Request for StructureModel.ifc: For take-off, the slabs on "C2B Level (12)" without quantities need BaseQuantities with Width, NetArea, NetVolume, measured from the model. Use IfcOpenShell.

First a look at what the model holds.

```python
import ifcopenshell
import ifcopenshell.util.element
import ifcopenshell.util.unit

model = ifcopenshell.open("StructureModel.ifc")
print(model.schema)
for unit_type in ("LENGTHUNIT", "AREAUNIT", "VOLUMEUNIT"):
    print(unit_type, ifcopenshell.util.unit.calculate_unit_scale(model, unit_type))
storey = next(s for s in model.by_type("IfcBuildingStorey") if s.Name == "C2B Level (12)")
slabs = [e for e in ifcopenshell.util.element.get_decomposition(storey) if e.is_a("IfcSlab")]
for e in sorted(slabs, key=lambda e: e.id()):
    print(e.id(), e.is_a(), e.Name, list(ifcopenshell.util.element.get_psets(e, qtos_only=True)), sep=" | ")
```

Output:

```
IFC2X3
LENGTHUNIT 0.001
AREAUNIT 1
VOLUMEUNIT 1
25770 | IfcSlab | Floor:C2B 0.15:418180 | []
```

```python
import ifcopenshell
import ifcopenshell.api.pset
import ifcopenshell.geom
import ifcopenshell.util.element
import ifcopenshell.util.shape
import ifcopenshell.util.unit

model = ifcopenshell.open("StructureModel.ifc")
unit_scale = ifcopenshell.util.unit.calculate_unit_scale(model)
area_scale = ifcopenshell.util.unit.calculate_unit_scale(model, "AREAUNIT")
volume_scale = ifcopenshell.util.unit.calculate_unit_scale(model, "VOLUMEUNIT")
settings = ifcopenshell.geom.settings()

storey = next(s for s in model.by_type("IfcBuildingStorey") if s.Name == "C2B Level (12)")
slabs = [e for e in ifcopenshell.util.element.get_decomposition(storey) if e.is_a("IfcSlab")]

for e in sorted(slabs, key=lambda e: e.id()):
    if ifcopenshell.util.element.get_psets(e, qtos_only=True, should_inherit=False):
        continue
    # Geometry comes back in metres, in the element's own axes.
    shape = ifcopenshell.geom.create_shape(settings, e)
    values = {
        "Width": ifcopenshell.util.shape.get_z(shape.geometry) / unit_scale,
        "NetArea": ifcopenshell.util.shape.get_footprint_area(shape.geometry) / area_scale,
        "NetVolume": ifcopenshell.util.shape.get_volume(shape.geometry) / volume_scale,
    }
    qto = ifcopenshell.api.pset.add_qto(model, product=e, name="BaseQuantities")
    ifcopenshell.api.pset.edit_qto(model, qto=qto, properties=values)
    print(e.id(), {k: round(v, 3) for k, v in values.items()})

model.write("StructureModel-out.ifc")
```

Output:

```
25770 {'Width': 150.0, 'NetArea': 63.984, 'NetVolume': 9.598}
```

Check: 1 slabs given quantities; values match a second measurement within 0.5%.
